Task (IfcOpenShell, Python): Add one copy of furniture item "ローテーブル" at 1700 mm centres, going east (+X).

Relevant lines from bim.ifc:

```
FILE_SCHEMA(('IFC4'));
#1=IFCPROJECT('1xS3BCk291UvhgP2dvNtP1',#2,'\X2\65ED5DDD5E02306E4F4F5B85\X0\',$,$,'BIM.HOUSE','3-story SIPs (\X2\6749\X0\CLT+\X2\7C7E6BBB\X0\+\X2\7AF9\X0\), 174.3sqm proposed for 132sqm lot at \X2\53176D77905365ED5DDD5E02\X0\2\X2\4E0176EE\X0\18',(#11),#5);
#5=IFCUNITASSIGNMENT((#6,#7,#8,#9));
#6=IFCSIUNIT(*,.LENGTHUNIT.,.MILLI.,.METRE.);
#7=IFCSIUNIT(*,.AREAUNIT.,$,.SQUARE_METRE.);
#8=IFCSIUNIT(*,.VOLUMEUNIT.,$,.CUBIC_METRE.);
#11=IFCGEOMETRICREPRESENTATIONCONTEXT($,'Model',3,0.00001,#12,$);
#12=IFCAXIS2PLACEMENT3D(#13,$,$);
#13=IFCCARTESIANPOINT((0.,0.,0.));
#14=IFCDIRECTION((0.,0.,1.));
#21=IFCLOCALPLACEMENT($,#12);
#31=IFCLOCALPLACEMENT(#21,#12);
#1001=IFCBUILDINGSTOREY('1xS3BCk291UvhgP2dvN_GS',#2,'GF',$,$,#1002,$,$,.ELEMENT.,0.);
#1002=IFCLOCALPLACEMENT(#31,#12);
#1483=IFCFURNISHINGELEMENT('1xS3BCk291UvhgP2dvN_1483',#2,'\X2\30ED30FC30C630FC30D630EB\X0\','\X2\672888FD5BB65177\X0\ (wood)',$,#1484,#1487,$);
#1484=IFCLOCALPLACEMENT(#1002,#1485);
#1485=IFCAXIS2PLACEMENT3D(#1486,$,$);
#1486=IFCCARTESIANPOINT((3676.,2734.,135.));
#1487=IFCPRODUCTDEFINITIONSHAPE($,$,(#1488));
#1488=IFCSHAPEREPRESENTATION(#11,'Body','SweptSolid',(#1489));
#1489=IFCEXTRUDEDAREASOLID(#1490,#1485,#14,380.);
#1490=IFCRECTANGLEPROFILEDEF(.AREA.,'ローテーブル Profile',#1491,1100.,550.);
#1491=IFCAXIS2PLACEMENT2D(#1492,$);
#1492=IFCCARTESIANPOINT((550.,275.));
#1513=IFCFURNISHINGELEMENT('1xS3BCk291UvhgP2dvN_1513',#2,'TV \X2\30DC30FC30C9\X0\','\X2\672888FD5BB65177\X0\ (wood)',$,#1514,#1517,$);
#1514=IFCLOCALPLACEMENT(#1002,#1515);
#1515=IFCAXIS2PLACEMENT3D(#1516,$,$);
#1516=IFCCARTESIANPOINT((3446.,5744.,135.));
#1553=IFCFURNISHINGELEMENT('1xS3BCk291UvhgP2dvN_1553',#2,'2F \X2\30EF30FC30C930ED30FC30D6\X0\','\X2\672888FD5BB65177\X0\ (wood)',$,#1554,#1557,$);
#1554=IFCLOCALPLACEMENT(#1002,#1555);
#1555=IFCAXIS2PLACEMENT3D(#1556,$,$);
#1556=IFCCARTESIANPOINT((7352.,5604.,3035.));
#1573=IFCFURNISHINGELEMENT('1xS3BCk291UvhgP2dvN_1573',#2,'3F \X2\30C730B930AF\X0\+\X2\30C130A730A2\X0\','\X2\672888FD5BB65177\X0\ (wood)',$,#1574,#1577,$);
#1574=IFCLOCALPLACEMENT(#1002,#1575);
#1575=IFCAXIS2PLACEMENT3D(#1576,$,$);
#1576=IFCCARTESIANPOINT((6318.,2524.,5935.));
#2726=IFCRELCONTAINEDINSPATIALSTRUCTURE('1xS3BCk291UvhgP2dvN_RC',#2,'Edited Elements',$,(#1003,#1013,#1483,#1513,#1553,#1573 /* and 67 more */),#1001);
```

```python
import numpy as np
import ifcopenshell
import ifcopenshell.api.geometry
import ifcopenshell.api.root
import ifcopenshell.util.element
import ifcopenshell.util.placement

model = ifcopenshell.open("bim.ifc")


def reuse_history(source, copy):
    """copy_class also copies each property set's owner history, people and application; keep the originals."""
    for rel in copy.IsDefinedBy:
        if rel.is_a("IfcRelDefinesByProperties") and (history := rel.RelatingPropertyDefinition.OwnerHistory):
            rel.RelatingPropertyDefinition.OwnerHistory = source.OwnerHistory
            ifcopenshell.util.element.remove_deep2(model, history)


source = model.by_guid("1xS3BCk291UvhgP2dvN_1483")
base = ifcopenshell.util.placement.get_local_placement(source.ObjectPlacement)
step = np.array([1.0, 0.0, 0.0]) * 1700.0

for i in range(1, 2):
    copy = ifcopenshell.api.root.copy_class(model, product=source)
    copy.Representation = ifcopenshell.util.element.copy_deep(
        model, source.Representation, exclude=["IfcGeometricRepresentationContext", "IfcRepresentationMap"]
    )
    reuse_history(source, copy)
    matrix = base.copy()
    matrix[:3, 3] += i * step
    print("added at", matrix[:3, 3].round(3) + 0.0)
    ifcopenshell.api.geometry.edit_object_placement(model, product=copy, matrix=matrix, is_si=False)

model.write("bim_rev.ifc")
```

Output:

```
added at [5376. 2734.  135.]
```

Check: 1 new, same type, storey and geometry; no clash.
